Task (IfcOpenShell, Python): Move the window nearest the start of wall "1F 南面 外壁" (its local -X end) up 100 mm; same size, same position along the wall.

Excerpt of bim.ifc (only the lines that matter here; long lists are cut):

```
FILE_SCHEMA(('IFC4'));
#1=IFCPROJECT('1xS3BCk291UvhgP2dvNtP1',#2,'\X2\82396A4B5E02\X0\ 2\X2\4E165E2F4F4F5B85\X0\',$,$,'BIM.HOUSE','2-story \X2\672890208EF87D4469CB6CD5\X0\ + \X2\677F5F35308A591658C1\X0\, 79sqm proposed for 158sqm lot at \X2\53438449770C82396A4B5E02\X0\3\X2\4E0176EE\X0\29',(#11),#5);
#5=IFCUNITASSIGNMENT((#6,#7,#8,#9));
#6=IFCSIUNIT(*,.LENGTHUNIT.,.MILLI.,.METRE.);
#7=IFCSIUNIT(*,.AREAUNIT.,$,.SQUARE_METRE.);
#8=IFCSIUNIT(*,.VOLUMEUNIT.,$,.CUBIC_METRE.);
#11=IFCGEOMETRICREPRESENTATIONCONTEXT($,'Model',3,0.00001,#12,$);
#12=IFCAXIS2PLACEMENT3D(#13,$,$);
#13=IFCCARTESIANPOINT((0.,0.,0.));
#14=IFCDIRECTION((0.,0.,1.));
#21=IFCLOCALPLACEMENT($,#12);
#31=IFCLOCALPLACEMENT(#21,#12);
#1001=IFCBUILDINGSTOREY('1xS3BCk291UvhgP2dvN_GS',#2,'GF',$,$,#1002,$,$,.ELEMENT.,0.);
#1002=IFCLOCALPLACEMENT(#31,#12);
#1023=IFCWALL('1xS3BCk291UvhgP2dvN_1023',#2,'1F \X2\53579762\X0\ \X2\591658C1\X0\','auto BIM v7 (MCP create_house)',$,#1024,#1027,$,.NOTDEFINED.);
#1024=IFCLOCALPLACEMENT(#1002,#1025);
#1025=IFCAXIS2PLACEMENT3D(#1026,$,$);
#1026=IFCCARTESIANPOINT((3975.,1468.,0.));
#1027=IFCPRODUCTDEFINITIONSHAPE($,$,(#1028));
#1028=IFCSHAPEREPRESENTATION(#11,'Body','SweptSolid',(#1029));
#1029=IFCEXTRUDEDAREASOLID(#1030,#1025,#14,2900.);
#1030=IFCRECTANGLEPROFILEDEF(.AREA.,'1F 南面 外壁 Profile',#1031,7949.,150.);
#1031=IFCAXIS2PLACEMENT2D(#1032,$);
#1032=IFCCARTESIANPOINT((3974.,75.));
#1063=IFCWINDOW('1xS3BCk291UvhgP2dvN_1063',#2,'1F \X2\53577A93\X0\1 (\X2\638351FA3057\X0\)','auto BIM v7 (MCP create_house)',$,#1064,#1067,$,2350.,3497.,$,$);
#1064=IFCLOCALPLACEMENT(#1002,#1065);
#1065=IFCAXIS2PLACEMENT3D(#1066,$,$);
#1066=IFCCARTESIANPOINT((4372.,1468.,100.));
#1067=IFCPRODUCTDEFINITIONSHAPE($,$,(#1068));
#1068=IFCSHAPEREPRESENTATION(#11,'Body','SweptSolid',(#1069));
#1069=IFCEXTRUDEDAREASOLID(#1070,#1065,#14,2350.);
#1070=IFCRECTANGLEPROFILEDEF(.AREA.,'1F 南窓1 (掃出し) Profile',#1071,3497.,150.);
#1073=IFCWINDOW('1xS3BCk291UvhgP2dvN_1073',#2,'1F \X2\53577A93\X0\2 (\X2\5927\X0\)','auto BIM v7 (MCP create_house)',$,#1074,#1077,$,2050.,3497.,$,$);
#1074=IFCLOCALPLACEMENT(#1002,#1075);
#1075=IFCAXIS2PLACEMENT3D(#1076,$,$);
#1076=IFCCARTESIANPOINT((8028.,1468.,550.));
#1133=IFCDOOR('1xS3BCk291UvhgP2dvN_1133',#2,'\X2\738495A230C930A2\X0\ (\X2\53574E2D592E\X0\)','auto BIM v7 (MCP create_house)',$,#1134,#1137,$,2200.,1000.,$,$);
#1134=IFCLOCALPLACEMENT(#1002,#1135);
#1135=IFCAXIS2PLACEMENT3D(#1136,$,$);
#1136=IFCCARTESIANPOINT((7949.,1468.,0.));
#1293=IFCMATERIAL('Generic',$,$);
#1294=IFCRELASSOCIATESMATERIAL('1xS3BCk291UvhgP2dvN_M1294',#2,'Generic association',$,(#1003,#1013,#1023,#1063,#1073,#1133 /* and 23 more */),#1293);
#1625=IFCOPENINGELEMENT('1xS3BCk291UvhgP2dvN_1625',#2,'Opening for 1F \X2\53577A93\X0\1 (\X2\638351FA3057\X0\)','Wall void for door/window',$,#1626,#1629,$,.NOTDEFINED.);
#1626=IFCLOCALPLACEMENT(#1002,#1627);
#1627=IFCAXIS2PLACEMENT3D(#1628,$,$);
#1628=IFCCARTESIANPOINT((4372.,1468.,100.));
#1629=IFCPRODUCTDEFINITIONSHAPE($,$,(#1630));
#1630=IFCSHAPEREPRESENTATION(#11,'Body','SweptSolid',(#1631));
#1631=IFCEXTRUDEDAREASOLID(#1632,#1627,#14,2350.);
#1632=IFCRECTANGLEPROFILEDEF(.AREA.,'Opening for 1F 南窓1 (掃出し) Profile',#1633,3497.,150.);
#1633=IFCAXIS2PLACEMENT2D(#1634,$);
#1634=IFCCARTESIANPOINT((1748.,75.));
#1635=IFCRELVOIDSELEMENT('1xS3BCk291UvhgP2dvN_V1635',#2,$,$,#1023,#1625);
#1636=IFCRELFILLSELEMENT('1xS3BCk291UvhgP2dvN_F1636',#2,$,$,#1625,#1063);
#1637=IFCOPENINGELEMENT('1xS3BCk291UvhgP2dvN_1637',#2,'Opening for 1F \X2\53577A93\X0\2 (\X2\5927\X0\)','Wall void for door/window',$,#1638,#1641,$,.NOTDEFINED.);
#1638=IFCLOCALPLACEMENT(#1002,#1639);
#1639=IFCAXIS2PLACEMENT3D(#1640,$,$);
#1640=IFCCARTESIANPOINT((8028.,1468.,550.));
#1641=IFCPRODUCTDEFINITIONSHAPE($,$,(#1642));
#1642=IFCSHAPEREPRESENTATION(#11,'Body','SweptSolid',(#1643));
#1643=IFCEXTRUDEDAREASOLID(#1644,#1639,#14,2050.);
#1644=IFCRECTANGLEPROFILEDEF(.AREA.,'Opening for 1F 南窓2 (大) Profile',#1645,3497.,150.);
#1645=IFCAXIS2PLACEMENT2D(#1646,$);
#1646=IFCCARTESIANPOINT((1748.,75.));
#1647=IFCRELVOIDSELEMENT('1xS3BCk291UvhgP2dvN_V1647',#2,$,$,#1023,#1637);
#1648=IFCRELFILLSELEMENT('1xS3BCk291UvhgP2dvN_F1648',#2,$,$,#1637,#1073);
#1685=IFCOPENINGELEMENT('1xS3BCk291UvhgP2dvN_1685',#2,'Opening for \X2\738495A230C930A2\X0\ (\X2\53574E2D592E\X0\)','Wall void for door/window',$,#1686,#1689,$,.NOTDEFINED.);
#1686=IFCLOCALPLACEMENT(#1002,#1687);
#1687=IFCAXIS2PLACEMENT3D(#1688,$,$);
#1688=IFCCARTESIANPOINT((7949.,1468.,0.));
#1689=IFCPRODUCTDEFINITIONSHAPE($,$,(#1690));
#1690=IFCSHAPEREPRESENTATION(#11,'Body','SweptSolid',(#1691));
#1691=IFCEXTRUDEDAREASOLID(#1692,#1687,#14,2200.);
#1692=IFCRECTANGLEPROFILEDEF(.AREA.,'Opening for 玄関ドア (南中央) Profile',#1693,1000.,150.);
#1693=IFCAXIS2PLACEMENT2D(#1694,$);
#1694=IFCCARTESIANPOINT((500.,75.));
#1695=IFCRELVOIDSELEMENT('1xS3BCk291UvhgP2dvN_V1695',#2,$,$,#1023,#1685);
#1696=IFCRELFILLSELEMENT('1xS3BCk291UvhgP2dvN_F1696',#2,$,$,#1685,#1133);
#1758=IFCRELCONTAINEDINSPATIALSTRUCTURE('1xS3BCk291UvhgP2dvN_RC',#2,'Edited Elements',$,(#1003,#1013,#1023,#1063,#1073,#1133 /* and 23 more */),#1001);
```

```python
import numpy as np
import ifcopenshell
import ifcopenshell.api.geometry
import ifcopenshell.util.placement
import ifcopenshell.util.unit

model = ifcopenshell.open("bim.ifc")
unit_scale = ifcopenshell.util.unit.calculate_unit_scale(model)

window = model.by_guid("1xS3BCk291UvhgP2dvN_1063")
opening = window.FillsVoids[0].RelatingOpeningElement
dz = 100.0

shift = np.array([0.0, 0.0, dz])
# The window is not placed relative to its opening, so move both.
for product in (opening, window):
    matrix = ifcopenshell.util.placement.get_local_placement(product.ObjectPlacement)
    matrix[:3, 3] += shift
    ifcopenshell.api.geometry.edit_object_placement(model, product=product, matrix=matrix, is_si=False)

print(f"moved by {dz * unit_scale:+.3f} m")

model.write("bim-out.ifc")
```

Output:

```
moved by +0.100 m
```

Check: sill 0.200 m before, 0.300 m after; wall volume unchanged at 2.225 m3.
